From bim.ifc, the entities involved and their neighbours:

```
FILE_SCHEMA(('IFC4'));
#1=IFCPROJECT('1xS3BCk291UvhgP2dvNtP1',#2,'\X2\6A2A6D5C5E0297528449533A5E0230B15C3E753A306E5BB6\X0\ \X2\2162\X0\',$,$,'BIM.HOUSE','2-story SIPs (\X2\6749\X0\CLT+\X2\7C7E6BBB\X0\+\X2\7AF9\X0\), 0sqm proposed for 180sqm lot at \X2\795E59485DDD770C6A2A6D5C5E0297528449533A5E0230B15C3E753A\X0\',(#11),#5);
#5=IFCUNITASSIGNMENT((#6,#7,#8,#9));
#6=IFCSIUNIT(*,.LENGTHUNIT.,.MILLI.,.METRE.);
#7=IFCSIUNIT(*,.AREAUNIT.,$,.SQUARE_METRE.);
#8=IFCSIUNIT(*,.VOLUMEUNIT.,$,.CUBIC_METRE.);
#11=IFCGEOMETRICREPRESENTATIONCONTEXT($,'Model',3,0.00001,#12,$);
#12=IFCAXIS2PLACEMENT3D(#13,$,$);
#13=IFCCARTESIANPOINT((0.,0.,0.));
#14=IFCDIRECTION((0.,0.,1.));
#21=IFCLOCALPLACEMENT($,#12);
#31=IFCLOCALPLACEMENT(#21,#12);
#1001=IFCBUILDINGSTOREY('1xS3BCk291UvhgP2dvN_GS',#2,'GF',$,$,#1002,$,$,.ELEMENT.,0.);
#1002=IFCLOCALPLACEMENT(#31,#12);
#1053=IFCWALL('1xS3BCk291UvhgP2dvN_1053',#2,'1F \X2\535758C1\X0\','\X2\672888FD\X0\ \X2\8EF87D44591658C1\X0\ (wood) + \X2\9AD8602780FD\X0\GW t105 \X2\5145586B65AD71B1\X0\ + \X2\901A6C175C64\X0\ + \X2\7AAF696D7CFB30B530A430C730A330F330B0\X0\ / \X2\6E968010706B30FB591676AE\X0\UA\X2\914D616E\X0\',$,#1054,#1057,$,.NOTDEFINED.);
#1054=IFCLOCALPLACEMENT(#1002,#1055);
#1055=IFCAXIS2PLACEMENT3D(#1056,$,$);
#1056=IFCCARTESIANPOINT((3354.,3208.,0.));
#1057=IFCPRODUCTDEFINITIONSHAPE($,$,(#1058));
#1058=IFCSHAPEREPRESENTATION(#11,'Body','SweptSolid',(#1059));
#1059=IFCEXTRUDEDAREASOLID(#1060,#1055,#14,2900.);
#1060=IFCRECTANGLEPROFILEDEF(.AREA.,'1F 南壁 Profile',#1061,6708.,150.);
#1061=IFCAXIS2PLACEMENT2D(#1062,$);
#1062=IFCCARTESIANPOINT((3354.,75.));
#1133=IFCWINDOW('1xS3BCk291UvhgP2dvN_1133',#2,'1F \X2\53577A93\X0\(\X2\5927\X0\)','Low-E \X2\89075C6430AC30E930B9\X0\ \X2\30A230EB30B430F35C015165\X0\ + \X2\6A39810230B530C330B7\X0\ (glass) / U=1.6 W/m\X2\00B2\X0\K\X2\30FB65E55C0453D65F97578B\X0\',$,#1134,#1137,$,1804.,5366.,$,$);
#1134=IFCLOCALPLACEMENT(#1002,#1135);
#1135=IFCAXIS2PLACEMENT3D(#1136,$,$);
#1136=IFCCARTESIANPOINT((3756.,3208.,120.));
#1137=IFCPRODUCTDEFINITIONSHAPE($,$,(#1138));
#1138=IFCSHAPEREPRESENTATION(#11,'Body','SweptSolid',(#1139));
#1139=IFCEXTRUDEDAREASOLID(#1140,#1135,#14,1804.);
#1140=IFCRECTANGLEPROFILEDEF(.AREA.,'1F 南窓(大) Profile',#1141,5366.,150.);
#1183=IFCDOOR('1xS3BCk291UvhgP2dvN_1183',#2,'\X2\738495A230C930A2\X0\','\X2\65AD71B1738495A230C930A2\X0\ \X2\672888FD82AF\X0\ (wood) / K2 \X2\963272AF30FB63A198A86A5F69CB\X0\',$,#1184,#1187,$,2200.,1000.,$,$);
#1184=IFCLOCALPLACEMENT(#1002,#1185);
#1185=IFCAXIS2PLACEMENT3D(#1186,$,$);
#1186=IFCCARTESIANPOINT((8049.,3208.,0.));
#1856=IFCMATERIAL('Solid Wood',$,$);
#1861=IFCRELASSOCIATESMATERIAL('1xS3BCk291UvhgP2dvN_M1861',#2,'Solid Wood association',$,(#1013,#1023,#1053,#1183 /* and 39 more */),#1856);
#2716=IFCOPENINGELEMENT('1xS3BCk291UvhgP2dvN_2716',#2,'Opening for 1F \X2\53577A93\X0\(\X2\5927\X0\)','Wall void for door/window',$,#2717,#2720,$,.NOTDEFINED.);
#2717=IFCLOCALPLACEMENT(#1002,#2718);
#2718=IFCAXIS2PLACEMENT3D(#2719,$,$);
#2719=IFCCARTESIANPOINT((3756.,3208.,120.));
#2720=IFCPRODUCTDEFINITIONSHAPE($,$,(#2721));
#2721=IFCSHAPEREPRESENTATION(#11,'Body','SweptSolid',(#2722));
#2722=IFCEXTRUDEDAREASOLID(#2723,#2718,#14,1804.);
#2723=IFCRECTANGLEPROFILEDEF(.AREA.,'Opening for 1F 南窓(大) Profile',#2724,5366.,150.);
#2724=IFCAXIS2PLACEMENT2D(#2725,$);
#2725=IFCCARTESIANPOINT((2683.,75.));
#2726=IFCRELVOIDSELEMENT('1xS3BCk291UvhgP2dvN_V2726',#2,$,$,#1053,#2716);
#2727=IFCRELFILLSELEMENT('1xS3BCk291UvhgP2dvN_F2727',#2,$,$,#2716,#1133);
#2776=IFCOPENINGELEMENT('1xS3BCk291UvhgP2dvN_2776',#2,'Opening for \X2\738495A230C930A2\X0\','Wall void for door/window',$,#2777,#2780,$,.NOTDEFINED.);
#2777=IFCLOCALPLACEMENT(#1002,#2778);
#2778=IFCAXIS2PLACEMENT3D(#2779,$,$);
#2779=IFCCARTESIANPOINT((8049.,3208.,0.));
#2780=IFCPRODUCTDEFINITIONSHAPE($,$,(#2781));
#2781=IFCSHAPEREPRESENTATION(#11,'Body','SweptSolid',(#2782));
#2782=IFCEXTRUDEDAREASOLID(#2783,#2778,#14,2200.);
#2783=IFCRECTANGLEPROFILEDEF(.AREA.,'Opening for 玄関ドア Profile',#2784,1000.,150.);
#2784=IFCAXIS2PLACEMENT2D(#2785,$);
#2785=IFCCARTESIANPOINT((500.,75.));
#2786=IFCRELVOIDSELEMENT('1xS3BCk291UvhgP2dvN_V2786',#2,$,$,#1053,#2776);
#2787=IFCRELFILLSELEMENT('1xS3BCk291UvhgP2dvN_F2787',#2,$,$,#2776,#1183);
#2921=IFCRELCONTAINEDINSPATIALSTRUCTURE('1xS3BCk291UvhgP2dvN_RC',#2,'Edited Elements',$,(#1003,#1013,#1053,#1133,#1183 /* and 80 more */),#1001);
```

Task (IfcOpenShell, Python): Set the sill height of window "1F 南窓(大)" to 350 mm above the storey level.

```python
import numpy as np
import ifcopenshell
import ifcopenshell.api.geometry
import ifcopenshell.geom
import ifcopenshell.util.element
import ifcopenshell.util.placement
import ifcopenshell.util.shape
import ifcopenshell.util.unit

model = ifcopenshell.open("bim.ifc")
unit_scale = ifcopenshell.util.unit.calculate_unit_scale(model)

window = model.by_guid("1xS3BCk291UvhgP2dvN_1133")
opening = window.FillsVoids[0].RelatingOpeningElement
storey = ifcopenshell.util.element.get_container(window, ifc_class="IfcBuildingStorey")
level = ifcopenshell.util.placement.get_local_placement(storey.ObjectPlacement)[2, 3]

# The opening's origin need not be at the sill, so measure its lowest point.
shape = ifcopenshell.geom.create_shape(ifcopenshell.geom.settings(), opening)
bottom = ifcopenshell.util.shape.get_shape_bottom_elevation(shape, shape.geometry) / unit_scale
dz = level + 0.35 / unit_scale - bottom

shift = np.array([0.0, 0.0, dz])
# The window is not placed relative to its opening, so move both.
for product in (opening, window):
    matrix = ifcopenshell.util.placement.get_local_placement(product.ObjectPlacement)
    matrix[:3, 3] += shift
    ifcopenshell.api.geometry.edit_object_placement(model, product=product, matrix=matrix, is_si=False)

print(f"moved by {dz * unit_scale:+.3f} m")

model.write("bim_updated.ifc")
```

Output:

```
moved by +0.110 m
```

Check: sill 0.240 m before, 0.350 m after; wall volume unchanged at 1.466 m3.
